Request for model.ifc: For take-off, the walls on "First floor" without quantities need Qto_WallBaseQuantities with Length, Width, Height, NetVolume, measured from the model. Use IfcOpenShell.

First a look at what the model holds.

```python
import ifcopenshell
import ifcopenshell.util.element
import ifcopenshell.util.unit

model = ifcopenshell.open("model.ifc")
print(model.schema)
for unit_type in ("LENGTHUNIT", "AREAUNIT", "VOLUMEUNIT"):
    print(unit_type, ifcopenshell.util.unit.calculate_unit_scale(model, unit_type))
storey = next(s for s in model.by_type("IfcBuildingStorey") if s.Name == "First floor")
walls = [e for e in ifcopenshell.util.element.get_decomposition(storey) if e.is_a("IfcWall")]
for e in sorted(walls, key=lambda e: e.id()):
    print(e.id(), e.is_a(), e.Name, list(ifcopenshell.util.element.get_psets(e, qtos_only=True)), sep=" | ")
```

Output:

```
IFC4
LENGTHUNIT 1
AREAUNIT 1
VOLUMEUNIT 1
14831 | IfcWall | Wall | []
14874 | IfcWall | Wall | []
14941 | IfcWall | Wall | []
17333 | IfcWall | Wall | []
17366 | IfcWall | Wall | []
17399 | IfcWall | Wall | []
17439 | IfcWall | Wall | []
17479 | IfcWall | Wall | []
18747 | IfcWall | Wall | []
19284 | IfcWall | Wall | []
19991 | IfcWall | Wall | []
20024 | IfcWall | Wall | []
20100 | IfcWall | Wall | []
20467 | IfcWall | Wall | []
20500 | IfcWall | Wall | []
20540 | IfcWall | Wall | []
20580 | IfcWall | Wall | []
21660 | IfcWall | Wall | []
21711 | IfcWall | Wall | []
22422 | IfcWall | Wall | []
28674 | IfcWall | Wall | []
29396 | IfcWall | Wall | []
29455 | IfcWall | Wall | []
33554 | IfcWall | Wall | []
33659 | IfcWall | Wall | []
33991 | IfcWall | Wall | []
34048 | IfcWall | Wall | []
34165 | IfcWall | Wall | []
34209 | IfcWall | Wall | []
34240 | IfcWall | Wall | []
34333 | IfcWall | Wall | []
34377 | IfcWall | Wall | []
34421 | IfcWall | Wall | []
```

```python
import ifcopenshell
import ifcopenshell.api.pset
import ifcopenshell.geom
import ifcopenshell.util.element
import ifcopenshell.util.shape
import ifcopenshell.util.unit

model = ifcopenshell.open("model.ifc")
unit_scale = ifcopenshell.util.unit.calculate_unit_scale(model)
volume_scale = ifcopenshell.util.unit.calculate_unit_scale(model, "VOLUMEUNIT")
settings = ifcopenshell.geom.settings()

storey = next(s for s in model.by_type("IfcBuildingStorey") if s.Name == "First floor")
walls = [e for e in ifcopenshell.util.element.get_decomposition(storey) if e.is_a("IfcWall")]

for e in sorted(walls, key=lambda e: e.id()):
    if ifcopenshell.util.element.get_psets(e, qtos_only=True, should_inherit=False):
        continue
    # Geometry comes back in metres, in the element's own axes.
    shape = ifcopenshell.geom.create_shape(settings, e)
    values = {
        "Length": ifcopenshell.util.shape.get_x(shape.geometry) / unit_scale,
        "Width": ifcopenshell.util.shape.get_y(shape.geometry) / unit_scale,
        "Height": ifcopenshell.util.shape.get_z(shape.geometry) / unit_scale,
        "NetVolume": ifcopenshell.util.shape.get_volume(shape.geometry) / volume_scale,
    }
    qto = ifcopenshell.api.pset.add_qto(model, product=e, name="Qto_WallBaseQuantities")
    ifcopenshell.api.pset.edit_qto(model, qto=qto, properties=values)
    print(e.id(), {k: round(v, 3) for k, v in values.items()})

model.write("model_edited.ifc")
```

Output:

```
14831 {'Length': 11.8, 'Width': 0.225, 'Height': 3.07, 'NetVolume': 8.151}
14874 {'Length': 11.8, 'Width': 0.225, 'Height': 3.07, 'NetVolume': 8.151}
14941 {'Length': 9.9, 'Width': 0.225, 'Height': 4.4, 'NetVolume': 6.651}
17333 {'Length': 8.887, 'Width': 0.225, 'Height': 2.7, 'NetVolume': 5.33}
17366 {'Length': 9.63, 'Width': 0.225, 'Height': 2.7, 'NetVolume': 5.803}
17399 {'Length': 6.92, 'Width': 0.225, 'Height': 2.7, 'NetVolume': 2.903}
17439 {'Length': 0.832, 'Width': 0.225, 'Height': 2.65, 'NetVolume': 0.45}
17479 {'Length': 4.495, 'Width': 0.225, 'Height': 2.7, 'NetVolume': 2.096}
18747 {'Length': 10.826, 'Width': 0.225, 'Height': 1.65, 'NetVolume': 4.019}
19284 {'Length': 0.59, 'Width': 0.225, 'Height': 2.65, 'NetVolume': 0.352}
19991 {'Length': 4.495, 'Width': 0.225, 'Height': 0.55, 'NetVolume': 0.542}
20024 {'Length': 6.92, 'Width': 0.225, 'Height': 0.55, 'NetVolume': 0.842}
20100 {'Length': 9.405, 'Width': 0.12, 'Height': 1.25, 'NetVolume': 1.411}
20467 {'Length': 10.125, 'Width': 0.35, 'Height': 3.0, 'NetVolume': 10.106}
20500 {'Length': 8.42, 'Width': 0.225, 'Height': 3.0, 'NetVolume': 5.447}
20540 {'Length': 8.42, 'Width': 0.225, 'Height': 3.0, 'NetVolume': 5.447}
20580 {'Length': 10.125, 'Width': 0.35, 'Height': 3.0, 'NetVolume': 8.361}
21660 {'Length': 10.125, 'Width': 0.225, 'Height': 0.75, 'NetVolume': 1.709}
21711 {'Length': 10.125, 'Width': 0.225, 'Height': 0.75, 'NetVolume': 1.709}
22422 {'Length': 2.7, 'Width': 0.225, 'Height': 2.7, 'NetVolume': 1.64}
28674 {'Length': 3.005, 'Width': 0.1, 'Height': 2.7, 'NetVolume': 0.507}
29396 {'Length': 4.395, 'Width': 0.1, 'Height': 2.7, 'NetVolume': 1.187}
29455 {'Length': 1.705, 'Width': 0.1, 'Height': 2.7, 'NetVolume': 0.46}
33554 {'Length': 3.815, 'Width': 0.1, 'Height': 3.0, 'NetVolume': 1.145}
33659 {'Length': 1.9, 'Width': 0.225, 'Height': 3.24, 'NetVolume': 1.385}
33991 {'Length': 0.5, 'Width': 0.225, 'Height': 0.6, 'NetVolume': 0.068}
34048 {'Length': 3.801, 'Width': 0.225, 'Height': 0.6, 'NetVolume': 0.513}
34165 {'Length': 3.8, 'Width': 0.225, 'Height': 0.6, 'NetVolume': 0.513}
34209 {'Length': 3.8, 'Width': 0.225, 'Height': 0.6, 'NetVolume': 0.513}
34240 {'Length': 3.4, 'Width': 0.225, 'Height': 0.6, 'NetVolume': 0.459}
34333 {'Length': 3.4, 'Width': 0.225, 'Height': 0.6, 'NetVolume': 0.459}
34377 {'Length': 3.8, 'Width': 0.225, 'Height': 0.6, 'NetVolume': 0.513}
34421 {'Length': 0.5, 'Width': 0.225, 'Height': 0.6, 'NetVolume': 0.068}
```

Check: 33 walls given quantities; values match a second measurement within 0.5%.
